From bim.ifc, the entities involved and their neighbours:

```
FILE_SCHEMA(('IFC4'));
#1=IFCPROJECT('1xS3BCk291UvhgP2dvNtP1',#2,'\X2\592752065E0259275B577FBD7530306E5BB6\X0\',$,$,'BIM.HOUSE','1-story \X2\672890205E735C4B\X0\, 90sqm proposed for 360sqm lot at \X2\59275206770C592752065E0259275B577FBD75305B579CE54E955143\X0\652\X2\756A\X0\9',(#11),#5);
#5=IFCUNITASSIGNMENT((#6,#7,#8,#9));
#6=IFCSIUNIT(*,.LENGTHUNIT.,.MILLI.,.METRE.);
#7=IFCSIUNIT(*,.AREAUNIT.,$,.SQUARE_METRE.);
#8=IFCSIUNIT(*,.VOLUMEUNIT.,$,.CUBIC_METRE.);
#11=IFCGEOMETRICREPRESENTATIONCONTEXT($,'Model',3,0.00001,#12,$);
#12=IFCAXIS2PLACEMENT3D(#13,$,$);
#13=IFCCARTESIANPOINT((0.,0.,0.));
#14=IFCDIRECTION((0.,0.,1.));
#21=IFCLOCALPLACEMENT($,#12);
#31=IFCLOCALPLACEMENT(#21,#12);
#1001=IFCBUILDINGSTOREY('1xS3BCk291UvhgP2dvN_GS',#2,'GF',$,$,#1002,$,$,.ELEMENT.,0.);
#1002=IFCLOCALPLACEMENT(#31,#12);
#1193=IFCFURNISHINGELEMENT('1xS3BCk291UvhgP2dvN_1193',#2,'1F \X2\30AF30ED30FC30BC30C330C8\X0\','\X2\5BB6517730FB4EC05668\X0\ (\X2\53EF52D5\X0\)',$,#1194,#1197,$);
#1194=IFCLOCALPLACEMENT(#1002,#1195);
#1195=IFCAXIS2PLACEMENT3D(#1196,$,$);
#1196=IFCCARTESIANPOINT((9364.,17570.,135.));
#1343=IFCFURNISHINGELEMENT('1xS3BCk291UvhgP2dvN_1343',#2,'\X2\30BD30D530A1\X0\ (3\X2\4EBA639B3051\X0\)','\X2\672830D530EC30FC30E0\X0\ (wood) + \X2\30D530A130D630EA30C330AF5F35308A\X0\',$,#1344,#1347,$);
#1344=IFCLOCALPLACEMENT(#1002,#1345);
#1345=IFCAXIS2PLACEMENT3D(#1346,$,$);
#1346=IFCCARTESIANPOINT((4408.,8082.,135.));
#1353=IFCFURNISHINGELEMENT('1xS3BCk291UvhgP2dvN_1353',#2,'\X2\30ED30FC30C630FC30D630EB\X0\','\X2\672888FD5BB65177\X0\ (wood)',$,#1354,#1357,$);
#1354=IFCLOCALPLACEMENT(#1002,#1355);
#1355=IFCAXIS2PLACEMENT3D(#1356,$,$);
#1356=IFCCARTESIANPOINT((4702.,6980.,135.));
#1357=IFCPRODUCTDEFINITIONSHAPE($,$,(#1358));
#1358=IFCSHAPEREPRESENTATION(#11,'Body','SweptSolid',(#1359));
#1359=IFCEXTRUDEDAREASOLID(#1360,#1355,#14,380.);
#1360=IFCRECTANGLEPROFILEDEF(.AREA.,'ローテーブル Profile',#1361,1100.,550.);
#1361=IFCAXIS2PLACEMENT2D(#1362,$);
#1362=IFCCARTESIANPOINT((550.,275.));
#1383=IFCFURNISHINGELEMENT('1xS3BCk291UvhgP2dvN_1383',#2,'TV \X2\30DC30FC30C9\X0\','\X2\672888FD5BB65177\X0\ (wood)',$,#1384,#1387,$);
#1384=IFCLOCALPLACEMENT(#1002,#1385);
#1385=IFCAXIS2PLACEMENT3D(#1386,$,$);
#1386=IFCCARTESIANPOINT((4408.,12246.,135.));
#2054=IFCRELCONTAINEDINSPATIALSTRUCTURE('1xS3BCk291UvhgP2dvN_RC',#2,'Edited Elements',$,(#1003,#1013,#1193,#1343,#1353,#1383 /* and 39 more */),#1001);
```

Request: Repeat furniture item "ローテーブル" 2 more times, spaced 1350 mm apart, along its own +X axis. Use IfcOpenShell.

```python
import ifcopenshell
import ifcopenshell.api.geometry
import ifcopenshell.api.root
import ifcopenshell.util.element
import ifcopenshell.util.placement

model = ifcopenshell.open("bim.ifc")


def reuse_history(source, copy):
    """copy_class also copies each property set's owner history, people and application; keep the originals."""
    for rel in copy.IsDefinedBy:
        if rel.is_a("IfcRelDefinesByProperties") and (history := rel.RelatingPropertyDefinition.OwnerHistory):
            rel.RelatingPropertyDefinition.OwnerHistory = source.OwnerHistory
            ifcopenshell.util.element.remove_deep2(model, history)


source = model.by_guid("1xS3BCk291UvhgP2dvN_1353")
base = ifcopenshell.util.placement.get_local_placement(source.ObjectPlacement)
step = base[:3, 0] * 1350.0

for i in range(1, 3):
    copy = ifcopenshell.api.root.copy_class(model, product=source)
    copy.Representation = ifcopenshell.util.element.copy_deep(
        model, source.Representation, exclude=["IfcGeometricRepresentationContext", "IfcRepresentationMap"]
    )
    reuse_history(source, copy)
    matrix = base.copy()
    matrix[:3, 3] += i * step
    print("added at", matrix[:3, 3].round(3) + 0.0)
    ifcopenshell.api.geometry.edit_object_placement(model, product=copy, matrix=matrix, is_si=False)

model.write("bim_updated.ifc")
```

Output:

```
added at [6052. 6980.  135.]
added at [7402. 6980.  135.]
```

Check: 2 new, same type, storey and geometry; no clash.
